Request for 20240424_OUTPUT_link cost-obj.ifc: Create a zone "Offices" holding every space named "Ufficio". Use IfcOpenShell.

First a look at what the model holds.

```python
import ifcopenshell

model = ifcopenshell.open("20240424_OUTPUT_link cost-obj.ifc")
print(model.schema)
seen = {}
for space in model.by_type("IfcSpace"):
    seen[space.LongName] = seen.get(space.LongName, 0) + 1
for name, count in sorted(seen.items(), key=str):
    print(count, "x", name)
print("zones:", [z.Name for z in model.by_type("IfcZone")][:20])
```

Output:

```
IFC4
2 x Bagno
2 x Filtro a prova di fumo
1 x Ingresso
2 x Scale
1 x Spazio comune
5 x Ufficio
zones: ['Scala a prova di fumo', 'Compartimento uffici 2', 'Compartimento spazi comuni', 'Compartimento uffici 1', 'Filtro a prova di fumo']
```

```python
import ifcopenshell
import ifcopenshell.api.group
import ifcopenshell.api.root

model = ifcopenshell.open("20240424_OUTPUT_link cost-obj.ifc")

names = {"Ufficio"}
spaces = [s for s in model.by_type("IfcSpace") if s.LongName in names]

zone = ifcopenshell.api.root.create_entity(model, ifc_class="IfcZone", name="Offices")
ifcopenshell.api.group.assign_group(model, products=spaces, group=zone)
print(len(spaces), "spaces in", zone.Name)

model.write("20240424_OUTPUT_link cost-obj_rev.ifc")
```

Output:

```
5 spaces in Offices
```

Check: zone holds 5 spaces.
